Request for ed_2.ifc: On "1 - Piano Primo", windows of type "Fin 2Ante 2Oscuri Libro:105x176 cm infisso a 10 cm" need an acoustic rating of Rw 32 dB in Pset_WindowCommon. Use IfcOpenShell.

First a look at what the model holds.

```python
import ifcopenshell
import ifcopenshell.util.element

model = ifcopenshell.open("ed_2.ifc")
print(model.schema)
storey = next(s for s in model.by_type("IfcBuildingStorey") if s.Name == "1 - Piano Primo")
windows = [e for e in ifcopenshell.util.element.get_decomposition(storey) if e.is_a("IfcWindow")]
seen = {}
for e in windows:
    element_type = ifcopenshell.util.element.get_type(e)
    key = (element_type.Name if element_type != e and element_type else None, ifcopenshell.util.element.get_pset(e, "Pset_WindowCommon", "AcousticRating"))
    seen[key] = seen.get(key, 0) + 1
for (name, value), count in sorted(seen.items(), key=str):
    print(count, "x", name, "|", value)
```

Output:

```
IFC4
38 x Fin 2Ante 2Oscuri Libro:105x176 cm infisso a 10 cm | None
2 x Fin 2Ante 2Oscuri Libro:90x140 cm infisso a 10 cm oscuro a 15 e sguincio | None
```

```python
import ifcopenshell
import ifcopenshell.api.pset
import ifcopenshell.util.element

model = ifcopenshell.open("ed_2.ifc")

storey = next(s for s in model.by_type("IfcBuildingStorey") if s.Name == "1 - Piano Primo")
windows = [e for e in ifcopenshell.util.element.get_decomposition(storey) if e.is_a("IfcWindow")]

count = 0
for e in windows:
    element_type = ifcopenshell.util.element.get_type(e)
    if element_type in (None, e) or element_type.Name != "Fin 2Ante 2Oscuri Libro:105x176 cm infisso a 10 cm":
        continue
    # add_pset returns the element's existing set when there is one.
    pset = ifcopenshell.api.pset.add_pset(model, product=e, name="Pset_WindowCommon")
    ifcopenshell.api.pset.edit_pset(model, pset=pset, properties={"AcousticRating": "Rw 32 dB"})
    count += 1

print(count, "windows updated")

model.write("ed_2_rev.ifc")
```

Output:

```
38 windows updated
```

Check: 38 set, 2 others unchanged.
